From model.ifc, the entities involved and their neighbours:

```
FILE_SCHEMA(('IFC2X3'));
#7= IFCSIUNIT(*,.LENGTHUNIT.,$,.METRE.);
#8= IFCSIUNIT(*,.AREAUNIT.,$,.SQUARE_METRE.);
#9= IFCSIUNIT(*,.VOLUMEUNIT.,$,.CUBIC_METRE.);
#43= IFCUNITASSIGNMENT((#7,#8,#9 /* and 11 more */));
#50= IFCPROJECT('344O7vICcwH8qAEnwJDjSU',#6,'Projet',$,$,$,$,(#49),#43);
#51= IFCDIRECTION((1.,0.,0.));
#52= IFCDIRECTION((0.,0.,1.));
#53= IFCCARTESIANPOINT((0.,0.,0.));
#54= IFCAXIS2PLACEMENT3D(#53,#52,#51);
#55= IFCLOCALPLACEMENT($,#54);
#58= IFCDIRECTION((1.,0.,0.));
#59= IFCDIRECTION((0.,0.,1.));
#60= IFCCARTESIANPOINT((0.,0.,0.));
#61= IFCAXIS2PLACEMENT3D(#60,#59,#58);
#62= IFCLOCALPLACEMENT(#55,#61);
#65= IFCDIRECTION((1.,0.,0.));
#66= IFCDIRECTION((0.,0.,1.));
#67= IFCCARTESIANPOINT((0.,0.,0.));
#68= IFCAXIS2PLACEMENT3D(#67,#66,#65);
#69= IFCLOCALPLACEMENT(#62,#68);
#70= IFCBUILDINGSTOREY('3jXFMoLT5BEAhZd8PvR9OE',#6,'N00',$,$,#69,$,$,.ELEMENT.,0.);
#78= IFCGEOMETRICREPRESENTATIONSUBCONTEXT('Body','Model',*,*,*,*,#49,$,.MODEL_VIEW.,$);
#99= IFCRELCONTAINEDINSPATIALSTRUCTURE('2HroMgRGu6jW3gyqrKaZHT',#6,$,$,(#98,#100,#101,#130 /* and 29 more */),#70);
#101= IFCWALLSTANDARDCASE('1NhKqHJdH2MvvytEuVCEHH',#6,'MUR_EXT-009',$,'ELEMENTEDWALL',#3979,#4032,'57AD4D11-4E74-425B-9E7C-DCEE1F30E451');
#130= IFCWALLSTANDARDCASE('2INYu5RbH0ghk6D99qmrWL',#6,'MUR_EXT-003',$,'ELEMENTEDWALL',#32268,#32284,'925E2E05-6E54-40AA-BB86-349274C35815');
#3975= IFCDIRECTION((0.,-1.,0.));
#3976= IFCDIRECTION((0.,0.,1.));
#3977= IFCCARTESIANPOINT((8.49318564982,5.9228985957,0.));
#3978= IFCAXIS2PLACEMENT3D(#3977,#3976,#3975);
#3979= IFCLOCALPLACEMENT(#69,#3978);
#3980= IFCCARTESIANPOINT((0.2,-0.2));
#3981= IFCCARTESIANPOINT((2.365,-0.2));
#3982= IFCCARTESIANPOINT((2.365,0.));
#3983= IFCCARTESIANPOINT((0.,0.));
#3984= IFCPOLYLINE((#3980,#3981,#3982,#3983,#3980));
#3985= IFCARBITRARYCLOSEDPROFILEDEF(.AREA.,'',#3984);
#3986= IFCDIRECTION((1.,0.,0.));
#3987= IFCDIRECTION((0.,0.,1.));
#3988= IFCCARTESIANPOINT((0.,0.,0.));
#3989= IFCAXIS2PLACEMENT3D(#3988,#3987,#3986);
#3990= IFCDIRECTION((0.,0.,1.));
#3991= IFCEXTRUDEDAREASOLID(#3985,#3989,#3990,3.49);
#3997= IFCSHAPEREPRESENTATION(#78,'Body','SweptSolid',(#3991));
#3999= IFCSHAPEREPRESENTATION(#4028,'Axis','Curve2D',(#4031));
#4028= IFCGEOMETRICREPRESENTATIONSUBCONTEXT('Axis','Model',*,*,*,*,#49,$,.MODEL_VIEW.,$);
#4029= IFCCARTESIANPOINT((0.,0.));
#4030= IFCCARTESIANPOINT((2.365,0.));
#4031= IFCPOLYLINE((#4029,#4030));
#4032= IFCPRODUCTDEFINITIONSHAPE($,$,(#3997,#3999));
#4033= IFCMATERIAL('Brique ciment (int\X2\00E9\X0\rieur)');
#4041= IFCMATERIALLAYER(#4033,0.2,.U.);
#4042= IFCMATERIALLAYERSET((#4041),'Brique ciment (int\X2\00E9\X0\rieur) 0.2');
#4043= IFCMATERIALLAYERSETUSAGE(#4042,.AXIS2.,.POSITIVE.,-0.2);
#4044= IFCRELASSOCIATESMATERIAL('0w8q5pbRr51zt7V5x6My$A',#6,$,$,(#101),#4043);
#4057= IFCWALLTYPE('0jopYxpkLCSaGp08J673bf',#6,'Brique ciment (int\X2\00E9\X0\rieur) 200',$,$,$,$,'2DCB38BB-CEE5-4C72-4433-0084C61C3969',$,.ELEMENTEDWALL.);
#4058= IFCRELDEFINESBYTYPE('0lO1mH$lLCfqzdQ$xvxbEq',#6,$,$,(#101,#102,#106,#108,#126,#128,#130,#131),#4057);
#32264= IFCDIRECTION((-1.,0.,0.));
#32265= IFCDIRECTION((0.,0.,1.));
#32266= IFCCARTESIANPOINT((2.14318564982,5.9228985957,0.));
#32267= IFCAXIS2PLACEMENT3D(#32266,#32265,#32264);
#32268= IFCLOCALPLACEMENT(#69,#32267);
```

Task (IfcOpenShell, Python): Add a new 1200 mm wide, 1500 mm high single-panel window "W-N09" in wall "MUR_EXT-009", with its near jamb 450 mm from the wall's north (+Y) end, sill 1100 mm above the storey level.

```python
import numpy as np
import ifcopenshell
import ifcopenshell.api.feature
import ifcopenshell.api.geometry
import ifcopenshell.api.root
import ifcopenshell.api.spatial
import ifcopenshell.api.type
import ifcopenshell.geom
import ifcopenshell.util.element
import ifcopenshell.util.placement
import ifcopenshell.util.representation
import ifcopenshell.util.shape
import ifcopenshell.util.unit

model = ifcopenshell.open("model.ifc")
unit_scale = ifcopenshell.util.unit.calculate_unit_scale(model)
settings = ifcopenshell.geom.settings()


def volume(element):
    """Net volume in cubic metres, openings subtracted."""
    shape = ifcopenshell.geom.create_shape(settings, element)
    return ifcopenshell.util.shape.get_volume(shape.geometry)


wall = model.by_guid("1NhKqHJdH2MvvytEuVCEHH")
storey = ifcopenshell.util.element.get_container(wall, ifc_class="IfcBuildingStorey")
context = ifcopenshell.util.representation.get_context(model, "Model", "Body", "MODEL_VIEW")
before = volume(wall)

width, height, from_end, sill = 1.2, 1.5, 0.45, 1.1  # metres

# The wall runs along its own X axis, and the end named is its -X end.
wall_shape = ifcopenshell.geom.create_shape(settings, wall)
x, y, z = ifcopenshell.util.shape.get_vertices(wall_shape.geometry).T
start = x.min() + from_end
face, thickness = float(y.min()), float(y.max() - y.min())
wall_matrix = ifcopenshell.util.placement.get_local_placement(wall.ObjectPlacement)
level = ifcopenshell.util.placement.get_local_placement(storey.ObjectPlacement)[2, 3]


def in_wall(x, y):
    """Placement at x, y metres in the wall's axes, at sill height."""
    matrix = wall_matrix.copy()
    matrix[:, 3] = wall_matrix @ np.array([x / unit_scale, y / unit_scale, 0.0, 1.0])
    matrix[2, 3] = level + sill / unit_scale
    return matrix


# Opening: a box that overshoots both wall faces by 50 mm.
opening = ifcopenshell.api.root.create_entity(model, ifc_class="IfcOpeningElement")
box = ifcopenshell.api.geometry.add_wall_representation(
    model, context=context, length=width, height=height, thickness=thickness + 0.1
)
ifcopenshell.api.geometry.assign_representation(model, product=opening, representation=box)
ifcopenshell.api.geometry.edit_object_placement(model, product=opening, matrix=in_wall(start, face - 0.05), is_si=False)
ifcopenshell.api.feature.add_feature(model, feature=opening, element=wall)

window = ifcopenshell.api.root.create_entity(model, ifc_class="IfcWindow", name="W-N09")
window.OverallWidth, window.OverallHeight = width / unit_scale, height / unit_scale
body = ifcopenshell.api.geometry.add_window_representation(
    model,
    context=context,
    overall_width=window.OverallWidth,
    overall_height=window.OverallHeight,
    partition_type="SINGLE_PANEL",
)
ifcopenshell.api.geometry.assign_representation(model, product=window, representation=body)
ifcopenshell.api.spatial.assign_container(model, products=[window], relating_structure=storey)
fills = ifcopenshell.api.feature.add_filling(model, opening=opening, element=window)
fills.OwnerHistory = window.OwnerHistory  # required in IFC2X3

# IFC2X3 keeps the operation on the window style.
style = ifcopenshell.api.root.create_entity(model, ifc_class="IfcWindowStyle", name="W-N09")
style.OperationType, style.ConstructionType = "SINGLE_PANEL", "NOTDEFINED"
style.ParameterTakesPrecedence = style.Sizeable = False
ifcopenshell.api.type.assign_type(model, related_objects=[window], relating_type=style)

# Centre the window in the wall's thickness.
ifcopenshell.api.geometry.edit_object_placement(model, product=window, matrix=in_wall(start, face), is_si=False)
window_shape = ifcopenshell.geom.create_shape(settings, window)
depth = ifcopenshell.util.shape.get_vertices(window_shape.geometry)[:, 1]
offset = face + thickness / 2 - (depth.min() + depth.max()) / 2
ifcopenshell.api.geometry.edit_object_placement(model, product=window, matrix=in_wall(start, offset), is_si=False)

after = volume(wall)

print(f"wall volume {before:.3f} -> {after:.3f} m3")

model.write("model_v2.ifc")
```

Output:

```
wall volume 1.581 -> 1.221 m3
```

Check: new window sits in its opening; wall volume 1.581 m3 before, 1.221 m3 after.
